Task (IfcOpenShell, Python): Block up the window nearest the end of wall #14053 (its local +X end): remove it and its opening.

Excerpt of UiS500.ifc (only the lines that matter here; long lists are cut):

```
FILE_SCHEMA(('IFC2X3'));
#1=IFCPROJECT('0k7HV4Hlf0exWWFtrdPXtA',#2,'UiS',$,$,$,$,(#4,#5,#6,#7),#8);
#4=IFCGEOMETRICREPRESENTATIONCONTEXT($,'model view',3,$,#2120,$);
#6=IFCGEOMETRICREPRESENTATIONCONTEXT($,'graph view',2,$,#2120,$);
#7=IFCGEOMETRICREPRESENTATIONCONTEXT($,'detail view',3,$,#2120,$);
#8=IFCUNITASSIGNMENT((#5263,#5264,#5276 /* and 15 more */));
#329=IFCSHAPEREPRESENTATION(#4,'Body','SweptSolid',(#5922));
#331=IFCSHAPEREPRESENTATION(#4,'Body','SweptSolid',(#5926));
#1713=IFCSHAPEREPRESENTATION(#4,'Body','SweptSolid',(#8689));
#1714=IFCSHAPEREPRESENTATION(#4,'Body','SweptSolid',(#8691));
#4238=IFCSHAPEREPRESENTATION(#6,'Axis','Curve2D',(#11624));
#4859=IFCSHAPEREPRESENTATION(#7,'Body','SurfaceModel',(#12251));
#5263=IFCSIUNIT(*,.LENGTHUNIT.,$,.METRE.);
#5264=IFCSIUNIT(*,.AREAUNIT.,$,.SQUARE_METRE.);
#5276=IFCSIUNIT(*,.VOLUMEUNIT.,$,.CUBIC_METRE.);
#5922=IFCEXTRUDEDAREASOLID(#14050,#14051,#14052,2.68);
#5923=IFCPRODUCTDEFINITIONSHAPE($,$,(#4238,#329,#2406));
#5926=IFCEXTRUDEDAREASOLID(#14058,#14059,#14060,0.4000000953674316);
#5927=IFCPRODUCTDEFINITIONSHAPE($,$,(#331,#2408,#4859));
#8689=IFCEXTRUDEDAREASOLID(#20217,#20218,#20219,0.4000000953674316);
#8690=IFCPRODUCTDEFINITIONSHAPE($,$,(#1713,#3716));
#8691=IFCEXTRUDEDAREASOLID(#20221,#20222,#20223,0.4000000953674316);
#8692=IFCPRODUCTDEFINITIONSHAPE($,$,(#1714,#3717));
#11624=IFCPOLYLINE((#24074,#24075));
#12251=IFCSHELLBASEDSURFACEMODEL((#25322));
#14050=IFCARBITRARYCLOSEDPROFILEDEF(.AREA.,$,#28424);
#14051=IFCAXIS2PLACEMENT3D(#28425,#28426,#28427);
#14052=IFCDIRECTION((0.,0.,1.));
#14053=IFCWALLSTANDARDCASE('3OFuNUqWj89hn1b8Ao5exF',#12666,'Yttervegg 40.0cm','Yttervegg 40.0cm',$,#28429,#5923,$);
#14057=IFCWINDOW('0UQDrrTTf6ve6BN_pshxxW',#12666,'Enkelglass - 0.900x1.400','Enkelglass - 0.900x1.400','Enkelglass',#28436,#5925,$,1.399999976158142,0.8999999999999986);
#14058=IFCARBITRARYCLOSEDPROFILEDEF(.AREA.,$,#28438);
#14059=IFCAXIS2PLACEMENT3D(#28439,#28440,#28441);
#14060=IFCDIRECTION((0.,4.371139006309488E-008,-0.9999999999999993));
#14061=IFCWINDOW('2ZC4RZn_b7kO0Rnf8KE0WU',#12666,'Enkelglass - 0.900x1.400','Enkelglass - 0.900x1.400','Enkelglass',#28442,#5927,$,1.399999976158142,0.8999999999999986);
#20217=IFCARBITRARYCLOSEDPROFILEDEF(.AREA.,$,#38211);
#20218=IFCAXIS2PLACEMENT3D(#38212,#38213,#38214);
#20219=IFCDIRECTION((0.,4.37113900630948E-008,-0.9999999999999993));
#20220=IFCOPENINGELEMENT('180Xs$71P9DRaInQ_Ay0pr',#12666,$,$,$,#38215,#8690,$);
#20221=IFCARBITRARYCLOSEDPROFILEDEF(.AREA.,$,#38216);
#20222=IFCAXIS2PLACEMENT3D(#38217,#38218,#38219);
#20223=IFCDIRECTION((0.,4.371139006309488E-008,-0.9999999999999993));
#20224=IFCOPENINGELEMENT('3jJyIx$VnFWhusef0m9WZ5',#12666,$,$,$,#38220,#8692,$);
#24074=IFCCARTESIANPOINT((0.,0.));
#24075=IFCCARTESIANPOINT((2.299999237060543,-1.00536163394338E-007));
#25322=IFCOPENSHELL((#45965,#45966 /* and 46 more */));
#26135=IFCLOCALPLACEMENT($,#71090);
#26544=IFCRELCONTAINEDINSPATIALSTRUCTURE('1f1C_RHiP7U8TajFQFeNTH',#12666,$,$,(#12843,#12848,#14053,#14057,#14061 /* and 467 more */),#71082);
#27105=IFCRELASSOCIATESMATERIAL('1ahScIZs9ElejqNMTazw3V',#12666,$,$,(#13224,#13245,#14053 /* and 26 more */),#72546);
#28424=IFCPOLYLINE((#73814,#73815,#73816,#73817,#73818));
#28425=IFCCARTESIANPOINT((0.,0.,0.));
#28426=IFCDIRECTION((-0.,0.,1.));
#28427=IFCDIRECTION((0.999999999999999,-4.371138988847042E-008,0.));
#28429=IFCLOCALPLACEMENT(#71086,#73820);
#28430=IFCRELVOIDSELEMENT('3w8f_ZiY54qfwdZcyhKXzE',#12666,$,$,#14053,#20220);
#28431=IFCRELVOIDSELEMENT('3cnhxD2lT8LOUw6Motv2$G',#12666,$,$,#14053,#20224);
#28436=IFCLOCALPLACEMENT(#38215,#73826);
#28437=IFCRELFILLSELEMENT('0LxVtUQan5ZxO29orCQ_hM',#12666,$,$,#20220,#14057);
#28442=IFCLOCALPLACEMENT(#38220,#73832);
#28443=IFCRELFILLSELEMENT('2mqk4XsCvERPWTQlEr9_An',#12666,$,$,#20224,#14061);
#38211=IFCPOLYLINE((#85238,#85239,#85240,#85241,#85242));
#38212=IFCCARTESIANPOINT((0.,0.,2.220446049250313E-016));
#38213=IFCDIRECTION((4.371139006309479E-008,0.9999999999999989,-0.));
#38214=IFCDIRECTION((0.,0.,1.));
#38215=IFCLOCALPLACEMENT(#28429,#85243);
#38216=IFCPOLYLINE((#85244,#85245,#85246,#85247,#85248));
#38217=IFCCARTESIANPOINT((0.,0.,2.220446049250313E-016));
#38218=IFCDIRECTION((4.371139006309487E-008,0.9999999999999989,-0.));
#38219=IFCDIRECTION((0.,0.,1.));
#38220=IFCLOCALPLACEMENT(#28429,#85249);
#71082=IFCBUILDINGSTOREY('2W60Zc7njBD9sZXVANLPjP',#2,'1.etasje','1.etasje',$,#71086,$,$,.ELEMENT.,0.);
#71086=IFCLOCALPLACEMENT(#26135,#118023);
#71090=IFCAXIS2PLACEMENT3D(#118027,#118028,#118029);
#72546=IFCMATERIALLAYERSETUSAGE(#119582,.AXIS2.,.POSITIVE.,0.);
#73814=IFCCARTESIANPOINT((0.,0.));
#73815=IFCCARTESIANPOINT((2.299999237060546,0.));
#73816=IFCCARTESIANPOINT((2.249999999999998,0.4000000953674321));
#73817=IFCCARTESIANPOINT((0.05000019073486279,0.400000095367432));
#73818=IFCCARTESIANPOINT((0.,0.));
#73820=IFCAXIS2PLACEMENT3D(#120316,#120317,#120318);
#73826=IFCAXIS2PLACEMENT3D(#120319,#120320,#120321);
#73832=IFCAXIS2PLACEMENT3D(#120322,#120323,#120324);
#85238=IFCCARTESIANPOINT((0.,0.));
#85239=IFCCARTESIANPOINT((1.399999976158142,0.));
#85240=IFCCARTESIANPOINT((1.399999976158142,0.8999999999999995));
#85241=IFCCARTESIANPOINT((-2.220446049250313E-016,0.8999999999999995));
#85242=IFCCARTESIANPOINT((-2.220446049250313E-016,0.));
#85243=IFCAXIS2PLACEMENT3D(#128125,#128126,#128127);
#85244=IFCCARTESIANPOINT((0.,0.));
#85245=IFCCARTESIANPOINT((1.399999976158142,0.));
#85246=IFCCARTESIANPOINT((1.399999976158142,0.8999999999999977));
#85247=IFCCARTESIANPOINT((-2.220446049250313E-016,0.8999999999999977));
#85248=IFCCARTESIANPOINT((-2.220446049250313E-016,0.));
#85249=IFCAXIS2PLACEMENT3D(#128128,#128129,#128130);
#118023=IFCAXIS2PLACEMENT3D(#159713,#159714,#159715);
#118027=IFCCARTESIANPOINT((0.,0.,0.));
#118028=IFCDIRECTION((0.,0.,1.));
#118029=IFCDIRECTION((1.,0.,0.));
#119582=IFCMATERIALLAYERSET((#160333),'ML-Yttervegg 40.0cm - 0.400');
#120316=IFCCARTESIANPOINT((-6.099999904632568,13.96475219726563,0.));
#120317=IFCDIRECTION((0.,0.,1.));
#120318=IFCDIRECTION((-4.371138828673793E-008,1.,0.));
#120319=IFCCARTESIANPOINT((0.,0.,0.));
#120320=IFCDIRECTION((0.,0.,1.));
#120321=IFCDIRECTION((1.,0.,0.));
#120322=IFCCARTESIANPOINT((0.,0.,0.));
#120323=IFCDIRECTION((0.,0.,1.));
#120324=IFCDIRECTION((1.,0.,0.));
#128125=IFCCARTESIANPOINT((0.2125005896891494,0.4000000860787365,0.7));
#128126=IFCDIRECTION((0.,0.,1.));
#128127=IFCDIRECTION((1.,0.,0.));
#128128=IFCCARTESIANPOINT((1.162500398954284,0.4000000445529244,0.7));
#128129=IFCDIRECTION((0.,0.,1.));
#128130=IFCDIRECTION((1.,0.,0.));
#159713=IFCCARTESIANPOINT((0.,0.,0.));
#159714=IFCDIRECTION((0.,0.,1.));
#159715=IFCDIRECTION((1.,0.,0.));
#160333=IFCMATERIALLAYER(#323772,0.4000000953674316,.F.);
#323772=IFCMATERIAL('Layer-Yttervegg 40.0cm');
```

```python
import ifcopenshell
import ifcopenshell.api.feature
import ifcopenshell.api.root
import ifcopenshell.geom
import ifcopenshell.util.shape

model = ifcopenshell.open("UiS500.ifc")
settings = ifcopenshell.geom.settings()


def volume(element):
    """Net volume in cubic metres, openings subtracted."""
    shape = ifcopenshell.geom.create_shape(settings, element)
    return ifcopenshell.util.shape.get_volume(shape.geometry)


window = model.by_guid("2ZC4RZn_b7kO0Rnf8KE0WU")
opening = window.FillsVoids[0].RelatingOpeningElement
wall = opening.VoidsElements[0].RelatingBuildingElement
before = volume(wall)

ifcopenshell.api.root.remove_product(model, product=window)
ifcopenshell.api.feature.remove_feature(model, feature=opening)

after = volume(wall)

print(f"wall volume {before:.3f} -> {after:.3f} m3")

model.write("UiS500-out.ifc")
```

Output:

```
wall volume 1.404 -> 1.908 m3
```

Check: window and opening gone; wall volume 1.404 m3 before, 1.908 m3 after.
